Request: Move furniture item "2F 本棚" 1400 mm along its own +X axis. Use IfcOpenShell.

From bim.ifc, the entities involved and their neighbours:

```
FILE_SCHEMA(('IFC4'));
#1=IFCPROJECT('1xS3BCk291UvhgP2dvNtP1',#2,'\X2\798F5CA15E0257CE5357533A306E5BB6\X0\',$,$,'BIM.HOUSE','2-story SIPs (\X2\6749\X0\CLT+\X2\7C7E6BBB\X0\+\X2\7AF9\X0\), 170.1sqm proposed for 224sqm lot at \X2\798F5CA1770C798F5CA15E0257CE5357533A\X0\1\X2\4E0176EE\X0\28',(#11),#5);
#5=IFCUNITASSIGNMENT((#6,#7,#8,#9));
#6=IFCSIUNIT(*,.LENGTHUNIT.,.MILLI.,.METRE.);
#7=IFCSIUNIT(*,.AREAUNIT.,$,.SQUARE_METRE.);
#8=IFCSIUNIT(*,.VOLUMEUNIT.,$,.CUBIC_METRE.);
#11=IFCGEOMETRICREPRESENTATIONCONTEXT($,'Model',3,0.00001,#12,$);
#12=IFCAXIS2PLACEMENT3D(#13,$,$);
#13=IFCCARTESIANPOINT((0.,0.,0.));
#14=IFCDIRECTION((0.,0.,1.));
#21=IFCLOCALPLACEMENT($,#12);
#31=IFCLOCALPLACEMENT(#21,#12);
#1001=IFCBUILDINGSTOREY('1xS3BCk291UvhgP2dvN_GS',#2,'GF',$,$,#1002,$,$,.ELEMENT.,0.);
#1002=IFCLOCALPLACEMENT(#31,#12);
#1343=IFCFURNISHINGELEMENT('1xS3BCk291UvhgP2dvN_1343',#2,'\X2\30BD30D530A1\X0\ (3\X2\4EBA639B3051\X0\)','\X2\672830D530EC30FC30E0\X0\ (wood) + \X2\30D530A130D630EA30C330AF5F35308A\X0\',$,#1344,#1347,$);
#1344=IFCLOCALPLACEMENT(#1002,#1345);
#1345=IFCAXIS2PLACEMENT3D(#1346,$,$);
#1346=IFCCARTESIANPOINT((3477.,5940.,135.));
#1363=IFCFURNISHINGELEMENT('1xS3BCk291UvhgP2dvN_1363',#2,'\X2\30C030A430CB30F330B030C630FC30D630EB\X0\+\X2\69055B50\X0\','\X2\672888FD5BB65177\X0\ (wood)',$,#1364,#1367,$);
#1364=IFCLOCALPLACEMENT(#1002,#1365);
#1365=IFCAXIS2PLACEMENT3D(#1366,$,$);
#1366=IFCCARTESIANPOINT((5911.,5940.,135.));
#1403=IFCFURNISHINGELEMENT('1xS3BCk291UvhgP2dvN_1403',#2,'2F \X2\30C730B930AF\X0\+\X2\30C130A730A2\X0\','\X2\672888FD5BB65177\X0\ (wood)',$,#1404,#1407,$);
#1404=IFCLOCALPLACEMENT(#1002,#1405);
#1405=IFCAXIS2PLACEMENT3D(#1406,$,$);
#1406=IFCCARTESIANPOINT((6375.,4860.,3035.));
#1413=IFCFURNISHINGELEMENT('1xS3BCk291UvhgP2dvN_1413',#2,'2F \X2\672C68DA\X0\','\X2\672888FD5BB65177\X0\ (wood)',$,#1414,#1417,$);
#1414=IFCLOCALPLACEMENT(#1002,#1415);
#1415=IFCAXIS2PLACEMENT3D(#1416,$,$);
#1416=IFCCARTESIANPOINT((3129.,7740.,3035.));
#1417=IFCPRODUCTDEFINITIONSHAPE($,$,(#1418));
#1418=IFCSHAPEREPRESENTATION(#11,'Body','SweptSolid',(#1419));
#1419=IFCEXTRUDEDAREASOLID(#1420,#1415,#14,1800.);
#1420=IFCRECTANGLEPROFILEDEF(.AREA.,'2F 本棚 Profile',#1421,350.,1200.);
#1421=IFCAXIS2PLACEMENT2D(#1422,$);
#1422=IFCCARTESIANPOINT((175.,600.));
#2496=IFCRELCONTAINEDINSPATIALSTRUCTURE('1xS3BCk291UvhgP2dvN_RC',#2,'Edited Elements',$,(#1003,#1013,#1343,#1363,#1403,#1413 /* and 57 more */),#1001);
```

```python
import ifcopenshell
import ifcopenshell.api.geometry
import ifcopenshell.util.placement
import ifcopenshell.util.unit

model = ifcopenshell.open("bim.ifc")
unit_scale = ifcopenshell.util.unit.calculate_unit_scale(model)

item = model.by_guid("1xS3BCk291UvhgP2dvN_1413")
matrix = ifcopenshell.util.placement.get_local_placement(item.ObjectPlacement)
matrix[:3, 3] += matrix[:3, 0] * 1.4 / unit_scale
ifcopenshell.api.geometry.edit_object_placement(model, product=item, matrix=matrix, is_si=False)

print(ifcopenshell.util.placement.get_local_placement(item.ObjectPlacement).round(3) + 0.0)

model.write("bim-out.ifc")
```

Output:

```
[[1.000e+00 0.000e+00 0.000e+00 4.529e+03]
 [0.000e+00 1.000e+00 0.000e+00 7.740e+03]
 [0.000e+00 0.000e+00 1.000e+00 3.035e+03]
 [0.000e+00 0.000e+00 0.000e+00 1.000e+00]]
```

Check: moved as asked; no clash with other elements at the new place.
